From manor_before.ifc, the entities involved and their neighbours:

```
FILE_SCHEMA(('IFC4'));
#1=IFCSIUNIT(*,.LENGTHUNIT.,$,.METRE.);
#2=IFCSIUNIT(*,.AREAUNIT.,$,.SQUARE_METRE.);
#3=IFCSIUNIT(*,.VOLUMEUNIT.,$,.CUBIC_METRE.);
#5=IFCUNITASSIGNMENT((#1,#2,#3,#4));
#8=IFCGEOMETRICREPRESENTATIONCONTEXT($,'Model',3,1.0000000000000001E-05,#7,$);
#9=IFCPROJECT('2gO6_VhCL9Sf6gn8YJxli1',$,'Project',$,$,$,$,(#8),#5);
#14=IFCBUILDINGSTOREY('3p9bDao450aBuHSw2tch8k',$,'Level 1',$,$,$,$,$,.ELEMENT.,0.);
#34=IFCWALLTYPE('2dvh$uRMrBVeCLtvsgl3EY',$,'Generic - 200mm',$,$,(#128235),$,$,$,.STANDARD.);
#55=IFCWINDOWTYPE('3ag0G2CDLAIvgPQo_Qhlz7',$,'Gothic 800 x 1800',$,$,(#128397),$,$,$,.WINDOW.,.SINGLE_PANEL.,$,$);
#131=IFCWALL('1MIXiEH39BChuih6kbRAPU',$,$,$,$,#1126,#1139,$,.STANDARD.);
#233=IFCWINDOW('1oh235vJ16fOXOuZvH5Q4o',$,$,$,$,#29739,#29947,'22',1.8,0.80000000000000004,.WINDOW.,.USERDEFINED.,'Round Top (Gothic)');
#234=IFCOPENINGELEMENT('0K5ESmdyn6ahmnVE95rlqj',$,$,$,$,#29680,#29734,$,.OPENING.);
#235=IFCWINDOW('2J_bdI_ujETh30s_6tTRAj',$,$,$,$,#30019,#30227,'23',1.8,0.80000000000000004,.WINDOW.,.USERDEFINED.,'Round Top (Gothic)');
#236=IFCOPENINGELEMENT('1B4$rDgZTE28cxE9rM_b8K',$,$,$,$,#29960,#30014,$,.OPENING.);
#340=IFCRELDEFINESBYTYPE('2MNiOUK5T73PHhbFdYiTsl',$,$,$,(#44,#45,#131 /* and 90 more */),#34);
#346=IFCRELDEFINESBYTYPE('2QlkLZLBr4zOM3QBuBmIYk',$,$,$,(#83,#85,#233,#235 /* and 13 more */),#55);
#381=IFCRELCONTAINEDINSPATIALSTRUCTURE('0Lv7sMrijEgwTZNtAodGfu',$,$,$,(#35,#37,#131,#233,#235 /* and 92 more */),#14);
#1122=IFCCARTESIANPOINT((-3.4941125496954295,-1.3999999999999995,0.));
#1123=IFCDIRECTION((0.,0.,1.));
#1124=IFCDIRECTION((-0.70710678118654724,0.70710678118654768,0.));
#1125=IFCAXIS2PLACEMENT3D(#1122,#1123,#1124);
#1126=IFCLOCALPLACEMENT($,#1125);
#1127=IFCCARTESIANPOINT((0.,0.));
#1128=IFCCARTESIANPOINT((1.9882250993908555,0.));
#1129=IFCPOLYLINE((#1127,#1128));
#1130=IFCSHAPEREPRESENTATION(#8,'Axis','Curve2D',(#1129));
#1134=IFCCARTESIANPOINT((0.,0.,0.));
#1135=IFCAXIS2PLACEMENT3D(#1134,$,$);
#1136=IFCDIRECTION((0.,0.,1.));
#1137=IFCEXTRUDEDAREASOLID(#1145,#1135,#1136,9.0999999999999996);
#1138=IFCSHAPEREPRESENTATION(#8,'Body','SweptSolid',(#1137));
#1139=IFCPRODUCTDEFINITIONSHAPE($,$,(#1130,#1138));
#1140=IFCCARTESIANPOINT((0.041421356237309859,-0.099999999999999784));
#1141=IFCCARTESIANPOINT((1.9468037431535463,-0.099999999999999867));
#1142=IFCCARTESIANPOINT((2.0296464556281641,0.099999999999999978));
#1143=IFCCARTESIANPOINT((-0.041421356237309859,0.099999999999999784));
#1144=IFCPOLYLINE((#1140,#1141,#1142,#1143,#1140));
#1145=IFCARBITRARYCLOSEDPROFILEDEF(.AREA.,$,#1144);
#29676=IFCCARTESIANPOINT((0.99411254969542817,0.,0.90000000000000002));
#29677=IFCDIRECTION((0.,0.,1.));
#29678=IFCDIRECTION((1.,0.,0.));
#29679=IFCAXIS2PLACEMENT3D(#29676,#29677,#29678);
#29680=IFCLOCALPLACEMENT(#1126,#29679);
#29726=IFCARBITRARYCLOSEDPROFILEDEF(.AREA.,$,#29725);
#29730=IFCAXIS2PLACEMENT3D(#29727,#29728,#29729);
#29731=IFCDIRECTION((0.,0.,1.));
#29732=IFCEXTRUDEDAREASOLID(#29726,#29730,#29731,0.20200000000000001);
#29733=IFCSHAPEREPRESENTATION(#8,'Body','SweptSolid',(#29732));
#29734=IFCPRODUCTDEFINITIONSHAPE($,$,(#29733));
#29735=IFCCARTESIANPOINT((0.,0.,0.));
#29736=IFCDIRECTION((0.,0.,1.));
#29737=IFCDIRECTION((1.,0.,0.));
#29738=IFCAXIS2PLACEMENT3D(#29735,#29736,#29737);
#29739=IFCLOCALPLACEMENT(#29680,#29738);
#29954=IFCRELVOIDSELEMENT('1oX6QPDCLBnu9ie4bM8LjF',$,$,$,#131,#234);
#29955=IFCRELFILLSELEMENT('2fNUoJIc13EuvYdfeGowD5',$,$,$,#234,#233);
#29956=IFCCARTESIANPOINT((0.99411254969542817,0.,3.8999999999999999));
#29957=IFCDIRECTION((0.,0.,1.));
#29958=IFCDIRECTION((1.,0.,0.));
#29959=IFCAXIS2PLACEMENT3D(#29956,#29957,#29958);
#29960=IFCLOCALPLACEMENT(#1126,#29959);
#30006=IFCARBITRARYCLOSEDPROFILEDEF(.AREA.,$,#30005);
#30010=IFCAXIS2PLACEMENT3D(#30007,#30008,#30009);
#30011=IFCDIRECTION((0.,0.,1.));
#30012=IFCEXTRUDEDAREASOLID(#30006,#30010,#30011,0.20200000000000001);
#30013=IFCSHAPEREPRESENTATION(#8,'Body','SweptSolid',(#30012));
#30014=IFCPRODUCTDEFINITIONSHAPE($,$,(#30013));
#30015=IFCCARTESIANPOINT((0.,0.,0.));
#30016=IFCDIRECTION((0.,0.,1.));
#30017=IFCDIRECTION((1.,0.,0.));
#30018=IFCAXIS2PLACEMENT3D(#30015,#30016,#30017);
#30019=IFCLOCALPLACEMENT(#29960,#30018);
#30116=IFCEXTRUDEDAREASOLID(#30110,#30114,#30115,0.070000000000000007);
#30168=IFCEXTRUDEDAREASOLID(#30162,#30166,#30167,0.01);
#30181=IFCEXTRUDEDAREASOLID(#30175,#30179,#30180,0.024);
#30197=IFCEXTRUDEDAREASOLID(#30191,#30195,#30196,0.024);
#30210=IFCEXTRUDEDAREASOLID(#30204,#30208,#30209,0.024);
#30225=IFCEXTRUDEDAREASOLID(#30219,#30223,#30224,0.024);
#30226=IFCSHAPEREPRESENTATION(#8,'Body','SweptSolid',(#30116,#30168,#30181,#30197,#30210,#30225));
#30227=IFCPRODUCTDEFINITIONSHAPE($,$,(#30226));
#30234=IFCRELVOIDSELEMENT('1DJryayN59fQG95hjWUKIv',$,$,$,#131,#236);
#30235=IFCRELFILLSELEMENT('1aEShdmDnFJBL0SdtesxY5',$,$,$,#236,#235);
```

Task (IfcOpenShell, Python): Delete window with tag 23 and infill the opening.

```python
import ifcopenshell
import ifcopenshell.api.feature
import ifcopenshell.api.root
import ifcopenshell.geom
import ifcopenshell.util.shape

model = ifcopenshell.open("manor_before.ifc")
settings = ifcopenshell.geom.settings()


def volume(element):
    """Net volume in cubic metres, openings subtracted."""
    shape = ifcopenshell.geom.create_shape(settings, element)
    return ifcopenshell.util.shape.get_volume(shape.geometry)


window = model.by_id(235)
opening = window.FillsVoids[0].RelatingOpeningElement
wall = opening.VoidsElements[0].RelatingBuildingElement
before = volume(wall)

ifcopenshell.api.root.remove_product(model, product=window)
ifcopenshell.api.feature.remove_feature(model, feature=opening)

after = volume(wall)

print(f"wall volume {before:.3f} -> {after:.3f} m3")

model.write("manor_before_rev.ifc")
```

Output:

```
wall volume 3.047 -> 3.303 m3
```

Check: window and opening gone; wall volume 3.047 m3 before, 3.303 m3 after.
